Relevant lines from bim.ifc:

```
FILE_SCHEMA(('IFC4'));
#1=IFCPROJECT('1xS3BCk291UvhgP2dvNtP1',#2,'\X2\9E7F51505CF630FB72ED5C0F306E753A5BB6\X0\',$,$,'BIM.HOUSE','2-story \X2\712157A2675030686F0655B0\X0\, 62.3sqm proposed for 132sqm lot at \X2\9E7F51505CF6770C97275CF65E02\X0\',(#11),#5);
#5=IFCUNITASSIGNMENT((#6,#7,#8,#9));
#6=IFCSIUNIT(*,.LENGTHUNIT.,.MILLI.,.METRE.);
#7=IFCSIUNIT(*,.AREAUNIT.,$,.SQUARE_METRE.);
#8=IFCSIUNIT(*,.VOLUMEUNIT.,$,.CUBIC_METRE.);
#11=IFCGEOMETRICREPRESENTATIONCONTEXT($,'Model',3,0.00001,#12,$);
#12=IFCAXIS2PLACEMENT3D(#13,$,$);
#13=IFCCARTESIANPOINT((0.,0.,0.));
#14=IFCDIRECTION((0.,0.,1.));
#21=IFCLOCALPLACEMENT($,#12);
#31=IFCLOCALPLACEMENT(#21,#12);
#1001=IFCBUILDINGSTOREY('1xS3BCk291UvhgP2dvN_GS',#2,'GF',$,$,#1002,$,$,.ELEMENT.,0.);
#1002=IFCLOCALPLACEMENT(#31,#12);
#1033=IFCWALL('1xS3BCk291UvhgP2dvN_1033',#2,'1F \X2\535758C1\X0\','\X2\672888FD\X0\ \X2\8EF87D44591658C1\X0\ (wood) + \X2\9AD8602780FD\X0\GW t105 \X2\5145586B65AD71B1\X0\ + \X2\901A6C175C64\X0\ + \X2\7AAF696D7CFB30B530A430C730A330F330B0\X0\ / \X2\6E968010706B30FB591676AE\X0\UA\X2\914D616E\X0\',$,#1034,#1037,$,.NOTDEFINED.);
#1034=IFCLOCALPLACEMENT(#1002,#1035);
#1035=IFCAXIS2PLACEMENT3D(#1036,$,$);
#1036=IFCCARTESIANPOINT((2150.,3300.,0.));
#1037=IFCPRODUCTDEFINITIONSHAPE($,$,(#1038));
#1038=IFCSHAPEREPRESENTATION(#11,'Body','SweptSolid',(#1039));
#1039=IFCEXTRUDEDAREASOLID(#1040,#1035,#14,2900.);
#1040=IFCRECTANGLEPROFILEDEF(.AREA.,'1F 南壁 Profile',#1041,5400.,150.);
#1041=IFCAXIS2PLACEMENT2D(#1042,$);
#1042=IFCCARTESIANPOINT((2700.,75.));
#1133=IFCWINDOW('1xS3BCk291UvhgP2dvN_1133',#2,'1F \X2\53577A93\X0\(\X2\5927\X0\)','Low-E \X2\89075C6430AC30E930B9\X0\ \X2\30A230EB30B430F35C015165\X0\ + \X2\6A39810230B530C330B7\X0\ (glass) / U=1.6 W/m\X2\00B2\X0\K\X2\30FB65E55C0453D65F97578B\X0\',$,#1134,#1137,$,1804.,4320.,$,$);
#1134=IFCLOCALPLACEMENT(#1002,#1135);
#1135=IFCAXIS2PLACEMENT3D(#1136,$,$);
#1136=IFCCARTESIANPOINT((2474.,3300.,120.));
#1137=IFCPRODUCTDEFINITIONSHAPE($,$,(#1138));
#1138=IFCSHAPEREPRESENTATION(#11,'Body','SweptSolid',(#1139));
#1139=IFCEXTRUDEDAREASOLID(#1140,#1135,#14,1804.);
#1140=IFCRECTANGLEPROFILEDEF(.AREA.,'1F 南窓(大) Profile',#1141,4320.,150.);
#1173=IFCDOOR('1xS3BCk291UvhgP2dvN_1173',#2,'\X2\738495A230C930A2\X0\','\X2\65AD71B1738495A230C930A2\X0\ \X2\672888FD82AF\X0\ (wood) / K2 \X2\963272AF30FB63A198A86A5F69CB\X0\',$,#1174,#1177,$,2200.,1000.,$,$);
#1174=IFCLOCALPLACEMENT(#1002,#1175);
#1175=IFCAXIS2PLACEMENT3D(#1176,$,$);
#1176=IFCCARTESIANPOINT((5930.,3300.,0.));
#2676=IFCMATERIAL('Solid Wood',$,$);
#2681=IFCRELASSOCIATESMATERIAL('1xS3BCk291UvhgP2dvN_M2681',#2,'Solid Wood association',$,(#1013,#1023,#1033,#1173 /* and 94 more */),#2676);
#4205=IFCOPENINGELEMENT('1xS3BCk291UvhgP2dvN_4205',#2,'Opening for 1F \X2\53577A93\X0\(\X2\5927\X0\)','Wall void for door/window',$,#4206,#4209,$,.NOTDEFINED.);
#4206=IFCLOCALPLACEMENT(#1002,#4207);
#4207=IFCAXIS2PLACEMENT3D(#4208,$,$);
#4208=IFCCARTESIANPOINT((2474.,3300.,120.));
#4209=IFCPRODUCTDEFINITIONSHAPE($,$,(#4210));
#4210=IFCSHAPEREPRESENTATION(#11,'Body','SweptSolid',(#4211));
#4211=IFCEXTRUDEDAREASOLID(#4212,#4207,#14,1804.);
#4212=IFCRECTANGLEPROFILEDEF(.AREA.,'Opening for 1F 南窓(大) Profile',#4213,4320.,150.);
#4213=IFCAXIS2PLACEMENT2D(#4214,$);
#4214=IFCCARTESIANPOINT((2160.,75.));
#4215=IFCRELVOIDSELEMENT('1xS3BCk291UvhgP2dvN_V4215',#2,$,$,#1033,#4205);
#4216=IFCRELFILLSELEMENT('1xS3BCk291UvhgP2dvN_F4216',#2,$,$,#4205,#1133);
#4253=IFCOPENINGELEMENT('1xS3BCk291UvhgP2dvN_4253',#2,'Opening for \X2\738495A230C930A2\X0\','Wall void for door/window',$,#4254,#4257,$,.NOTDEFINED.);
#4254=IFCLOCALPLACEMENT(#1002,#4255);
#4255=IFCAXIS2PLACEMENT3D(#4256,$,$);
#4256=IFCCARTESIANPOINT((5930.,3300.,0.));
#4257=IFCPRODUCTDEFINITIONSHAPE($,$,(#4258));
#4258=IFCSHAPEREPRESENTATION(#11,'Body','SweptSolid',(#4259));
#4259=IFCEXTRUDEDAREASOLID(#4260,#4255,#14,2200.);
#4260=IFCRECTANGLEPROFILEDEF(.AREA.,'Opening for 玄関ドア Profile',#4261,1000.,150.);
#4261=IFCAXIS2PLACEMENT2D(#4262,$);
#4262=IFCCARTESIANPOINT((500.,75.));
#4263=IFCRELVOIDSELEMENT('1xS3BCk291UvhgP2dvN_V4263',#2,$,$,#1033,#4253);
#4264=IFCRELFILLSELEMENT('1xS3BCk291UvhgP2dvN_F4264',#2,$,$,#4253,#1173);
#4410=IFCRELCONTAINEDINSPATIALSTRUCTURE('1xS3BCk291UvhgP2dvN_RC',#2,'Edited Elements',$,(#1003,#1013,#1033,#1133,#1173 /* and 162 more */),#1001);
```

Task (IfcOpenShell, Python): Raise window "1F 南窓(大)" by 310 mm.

```python
import numpy as np
import ifcopenshell
import ifcopenshell.api.geometry
import ifcopenshell.util.placement
import ifcopenshell.util.unit

model = ifcopenshell.open("bim.ifc")
unit_scale = ifcopenshell.util.unit.calculate_unit_scale(model)

window = model.by_guid("1xS3BCk291UvhgP2dvN_1133")
opening = window.FillsVoids[0].RelatingOpeningElement
dz = 0.31 / unit_scale

shift = np.array([0.0, 0.0, dz])
# The window is not placed relative to its opening, so move both.
for product in (opening, window):
    matrix = ifcopenshell.util.placement.get_local_placement(product.ObjectPlacement)
    matrix[:3, 3] += shift
    ifcopenshell.api.geometry.edit_object_placement(model, product=product, matrix=matrix, is_si=False)

print(f"moved by {dz * unit_scale:+.3f} m")

model.write("bim-out.ifc")
```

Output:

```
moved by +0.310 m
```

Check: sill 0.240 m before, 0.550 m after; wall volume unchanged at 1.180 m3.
